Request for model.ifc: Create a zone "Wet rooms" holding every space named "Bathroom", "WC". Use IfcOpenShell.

First a look at what the model holds.

```python
import ifcopenshell

model = ifcopenshell.open("model.ifc")
print(model.schema)
seen = {}
for space in model.by_type("IfcSpace"):
    seen[space.LongName] = seen.get(space.LongName, 0) + 1
for name, count in sorted(seen.items(), key=str):
    print(count, "x", name)
print("zones:", [z.Name for z in model.by_type("IfcZone")][:20])
```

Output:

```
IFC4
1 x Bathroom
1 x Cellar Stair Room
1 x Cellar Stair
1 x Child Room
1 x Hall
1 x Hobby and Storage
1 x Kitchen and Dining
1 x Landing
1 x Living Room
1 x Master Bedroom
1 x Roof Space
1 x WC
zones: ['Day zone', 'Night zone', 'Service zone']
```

```python
import ifcopenshell
import ifcopenshell.api.group
import ifcopenshell.api.root

model = ifcopenshell.open("model.ifc")

names = {"Bathroom", "WC"}
spaces = [s for s in model.by_type("IfcSpace") if s.LongName in names]

zone = ifcopenshell.api.root.create_entity(model, ifc_class="IfcZone", name="Wet rooms")
ifcopenshell.api.group.assign_group(model, products=spaces, group=zone)
print(len(spaces), "spaces in", zone.Name)

model.write("model_updated.ifc")
```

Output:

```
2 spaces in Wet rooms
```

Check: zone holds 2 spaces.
